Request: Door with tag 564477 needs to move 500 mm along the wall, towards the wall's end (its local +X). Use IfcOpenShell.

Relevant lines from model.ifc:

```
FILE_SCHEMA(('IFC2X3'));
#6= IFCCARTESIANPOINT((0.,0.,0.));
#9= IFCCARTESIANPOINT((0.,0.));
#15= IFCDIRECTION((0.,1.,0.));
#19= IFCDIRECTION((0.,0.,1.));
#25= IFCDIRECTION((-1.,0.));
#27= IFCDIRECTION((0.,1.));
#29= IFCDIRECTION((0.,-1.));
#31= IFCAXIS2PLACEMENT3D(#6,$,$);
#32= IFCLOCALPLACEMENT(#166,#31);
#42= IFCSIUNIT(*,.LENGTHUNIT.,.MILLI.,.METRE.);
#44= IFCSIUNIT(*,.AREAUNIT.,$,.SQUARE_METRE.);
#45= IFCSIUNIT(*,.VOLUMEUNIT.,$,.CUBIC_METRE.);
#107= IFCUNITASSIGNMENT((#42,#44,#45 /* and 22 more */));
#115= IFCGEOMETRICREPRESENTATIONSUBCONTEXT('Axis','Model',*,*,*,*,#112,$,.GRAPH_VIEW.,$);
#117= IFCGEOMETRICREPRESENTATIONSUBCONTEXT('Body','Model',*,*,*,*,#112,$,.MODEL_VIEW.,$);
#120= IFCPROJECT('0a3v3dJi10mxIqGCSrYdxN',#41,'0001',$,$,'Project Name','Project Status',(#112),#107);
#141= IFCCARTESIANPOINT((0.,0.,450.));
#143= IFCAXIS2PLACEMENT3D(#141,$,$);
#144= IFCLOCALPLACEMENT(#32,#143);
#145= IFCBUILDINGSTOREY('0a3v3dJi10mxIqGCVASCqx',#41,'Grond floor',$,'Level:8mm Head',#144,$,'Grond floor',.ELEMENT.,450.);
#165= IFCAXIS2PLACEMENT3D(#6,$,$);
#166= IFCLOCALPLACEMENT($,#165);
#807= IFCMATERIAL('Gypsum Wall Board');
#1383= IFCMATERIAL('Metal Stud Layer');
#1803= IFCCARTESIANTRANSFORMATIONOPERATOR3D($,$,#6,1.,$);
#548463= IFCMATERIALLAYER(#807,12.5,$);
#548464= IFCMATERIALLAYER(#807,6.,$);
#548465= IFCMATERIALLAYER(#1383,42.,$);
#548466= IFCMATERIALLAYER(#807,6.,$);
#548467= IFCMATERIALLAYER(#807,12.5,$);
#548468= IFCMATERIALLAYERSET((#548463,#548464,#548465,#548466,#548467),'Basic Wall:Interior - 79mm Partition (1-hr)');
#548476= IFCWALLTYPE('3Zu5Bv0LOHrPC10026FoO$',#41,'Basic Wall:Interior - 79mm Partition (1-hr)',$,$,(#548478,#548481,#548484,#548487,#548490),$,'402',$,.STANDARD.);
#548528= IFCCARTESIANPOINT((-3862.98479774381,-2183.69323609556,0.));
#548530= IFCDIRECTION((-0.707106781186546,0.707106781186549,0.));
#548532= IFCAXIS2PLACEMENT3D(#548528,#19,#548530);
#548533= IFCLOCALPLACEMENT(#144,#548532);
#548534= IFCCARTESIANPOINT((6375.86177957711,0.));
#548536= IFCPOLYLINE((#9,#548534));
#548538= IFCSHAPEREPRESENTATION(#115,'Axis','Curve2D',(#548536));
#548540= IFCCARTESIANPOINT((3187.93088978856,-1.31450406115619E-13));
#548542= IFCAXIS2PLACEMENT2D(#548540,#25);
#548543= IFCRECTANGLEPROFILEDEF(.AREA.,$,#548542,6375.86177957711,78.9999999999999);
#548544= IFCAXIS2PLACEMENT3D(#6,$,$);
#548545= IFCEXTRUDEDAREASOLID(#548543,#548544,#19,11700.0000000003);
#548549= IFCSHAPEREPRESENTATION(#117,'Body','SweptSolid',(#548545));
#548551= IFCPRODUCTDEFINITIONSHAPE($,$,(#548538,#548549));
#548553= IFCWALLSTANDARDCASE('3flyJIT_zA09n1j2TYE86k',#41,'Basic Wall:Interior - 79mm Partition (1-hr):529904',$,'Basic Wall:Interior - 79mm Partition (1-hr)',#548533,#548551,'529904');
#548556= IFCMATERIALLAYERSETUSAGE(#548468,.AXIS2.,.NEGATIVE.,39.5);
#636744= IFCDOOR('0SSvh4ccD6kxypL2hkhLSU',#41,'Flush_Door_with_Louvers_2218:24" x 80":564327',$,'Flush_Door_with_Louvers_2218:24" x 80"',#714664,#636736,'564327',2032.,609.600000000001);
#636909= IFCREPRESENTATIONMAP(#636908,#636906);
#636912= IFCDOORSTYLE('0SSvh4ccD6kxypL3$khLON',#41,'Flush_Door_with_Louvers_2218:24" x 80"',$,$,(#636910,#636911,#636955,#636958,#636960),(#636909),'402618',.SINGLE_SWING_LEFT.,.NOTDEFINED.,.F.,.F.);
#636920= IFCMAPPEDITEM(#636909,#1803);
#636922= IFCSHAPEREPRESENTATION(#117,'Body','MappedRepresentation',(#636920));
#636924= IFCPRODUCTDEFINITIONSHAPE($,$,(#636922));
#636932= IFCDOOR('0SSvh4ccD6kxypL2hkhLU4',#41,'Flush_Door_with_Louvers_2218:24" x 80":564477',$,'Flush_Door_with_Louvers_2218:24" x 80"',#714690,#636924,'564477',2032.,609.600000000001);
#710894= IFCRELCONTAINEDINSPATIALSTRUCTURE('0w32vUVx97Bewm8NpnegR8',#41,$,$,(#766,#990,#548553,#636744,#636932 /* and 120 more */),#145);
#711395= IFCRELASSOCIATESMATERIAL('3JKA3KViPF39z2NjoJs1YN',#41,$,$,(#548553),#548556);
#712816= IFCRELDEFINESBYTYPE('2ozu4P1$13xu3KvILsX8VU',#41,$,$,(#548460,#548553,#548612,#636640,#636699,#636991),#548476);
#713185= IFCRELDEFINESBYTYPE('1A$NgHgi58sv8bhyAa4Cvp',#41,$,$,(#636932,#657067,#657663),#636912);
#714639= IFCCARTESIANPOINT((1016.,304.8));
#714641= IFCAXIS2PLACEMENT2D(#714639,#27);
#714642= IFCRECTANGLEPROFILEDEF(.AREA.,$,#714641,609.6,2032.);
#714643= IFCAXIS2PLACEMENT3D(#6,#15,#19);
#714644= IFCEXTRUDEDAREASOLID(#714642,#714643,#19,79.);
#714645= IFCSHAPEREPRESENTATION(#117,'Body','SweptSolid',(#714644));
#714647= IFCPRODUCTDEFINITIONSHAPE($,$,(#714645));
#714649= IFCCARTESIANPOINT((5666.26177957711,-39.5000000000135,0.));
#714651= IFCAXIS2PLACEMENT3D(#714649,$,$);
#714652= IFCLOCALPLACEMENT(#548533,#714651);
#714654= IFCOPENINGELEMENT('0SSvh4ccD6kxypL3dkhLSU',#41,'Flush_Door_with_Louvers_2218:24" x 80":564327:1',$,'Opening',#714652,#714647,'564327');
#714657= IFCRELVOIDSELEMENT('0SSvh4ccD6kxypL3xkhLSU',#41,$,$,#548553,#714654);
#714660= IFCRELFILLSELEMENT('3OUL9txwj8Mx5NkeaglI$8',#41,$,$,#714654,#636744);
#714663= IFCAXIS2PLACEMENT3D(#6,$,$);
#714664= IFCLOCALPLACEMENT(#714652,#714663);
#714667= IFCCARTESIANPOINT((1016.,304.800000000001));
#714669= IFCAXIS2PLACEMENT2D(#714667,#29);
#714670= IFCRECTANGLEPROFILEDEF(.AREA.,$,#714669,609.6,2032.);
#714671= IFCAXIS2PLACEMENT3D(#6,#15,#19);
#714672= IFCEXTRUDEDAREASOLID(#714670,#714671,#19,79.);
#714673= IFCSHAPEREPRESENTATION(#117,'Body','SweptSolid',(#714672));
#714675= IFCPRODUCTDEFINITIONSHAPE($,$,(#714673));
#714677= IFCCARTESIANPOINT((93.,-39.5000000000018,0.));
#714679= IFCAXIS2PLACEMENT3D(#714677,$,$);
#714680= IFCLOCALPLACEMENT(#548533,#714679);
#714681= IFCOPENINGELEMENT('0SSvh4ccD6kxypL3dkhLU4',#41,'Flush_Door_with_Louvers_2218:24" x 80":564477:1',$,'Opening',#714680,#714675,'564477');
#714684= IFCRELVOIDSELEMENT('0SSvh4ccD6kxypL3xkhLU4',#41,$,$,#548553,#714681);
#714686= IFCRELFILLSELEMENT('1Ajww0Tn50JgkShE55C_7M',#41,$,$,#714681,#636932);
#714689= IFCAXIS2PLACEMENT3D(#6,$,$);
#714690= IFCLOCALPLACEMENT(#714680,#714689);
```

```python
import ifcopenshell
import ifcopenshell.api.geometry
import ifcopenshell.util.placement
import ifcopenshell.util.unit

model = ifcopenshell.open("model.ifc")
unit_scale = ifcopenshell.util.unit.calculate_unit_scale(model)

door = model.by_guid("0SSvh4ccD6kxypL2hkhLU4")
opening = door.FillsVoids[0].RelatingOpeningElement
wall = opening.VoidsElements[0].RelatingBuildingElement

wall_matrix = ifcopenshell.util.placement.get_local_placement(wall.ObjectPlacement)
shift = wall_matrix[:3, 0] * 0.5 / unit_scale
before = ifcopenshell.util.placement.get_local_placement(door.ObjectPlacement)[:3, 3].copy()

# The door is placed relative to its opening, so it follows when the opening moves.
matrix = ifcopenshell.util.placement.get_local_placement(opening.ObjectPlacement)
matrix[:3, 3] += shift
ifcopenshell.api.geometry.edit_object_placement(
    model, product=opening, matrix=matrix, is_si=False, should_transform_children=True
)

after = ifcopenshell.util.placement.get_local_placement(door.ObjectPlacement)[:3, 3]
print("door moved by", (after - before).round(3) + 0.0)

model.write("model_v2.ifc")
```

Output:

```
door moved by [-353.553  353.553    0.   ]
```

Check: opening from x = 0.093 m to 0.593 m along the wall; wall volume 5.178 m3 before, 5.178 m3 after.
